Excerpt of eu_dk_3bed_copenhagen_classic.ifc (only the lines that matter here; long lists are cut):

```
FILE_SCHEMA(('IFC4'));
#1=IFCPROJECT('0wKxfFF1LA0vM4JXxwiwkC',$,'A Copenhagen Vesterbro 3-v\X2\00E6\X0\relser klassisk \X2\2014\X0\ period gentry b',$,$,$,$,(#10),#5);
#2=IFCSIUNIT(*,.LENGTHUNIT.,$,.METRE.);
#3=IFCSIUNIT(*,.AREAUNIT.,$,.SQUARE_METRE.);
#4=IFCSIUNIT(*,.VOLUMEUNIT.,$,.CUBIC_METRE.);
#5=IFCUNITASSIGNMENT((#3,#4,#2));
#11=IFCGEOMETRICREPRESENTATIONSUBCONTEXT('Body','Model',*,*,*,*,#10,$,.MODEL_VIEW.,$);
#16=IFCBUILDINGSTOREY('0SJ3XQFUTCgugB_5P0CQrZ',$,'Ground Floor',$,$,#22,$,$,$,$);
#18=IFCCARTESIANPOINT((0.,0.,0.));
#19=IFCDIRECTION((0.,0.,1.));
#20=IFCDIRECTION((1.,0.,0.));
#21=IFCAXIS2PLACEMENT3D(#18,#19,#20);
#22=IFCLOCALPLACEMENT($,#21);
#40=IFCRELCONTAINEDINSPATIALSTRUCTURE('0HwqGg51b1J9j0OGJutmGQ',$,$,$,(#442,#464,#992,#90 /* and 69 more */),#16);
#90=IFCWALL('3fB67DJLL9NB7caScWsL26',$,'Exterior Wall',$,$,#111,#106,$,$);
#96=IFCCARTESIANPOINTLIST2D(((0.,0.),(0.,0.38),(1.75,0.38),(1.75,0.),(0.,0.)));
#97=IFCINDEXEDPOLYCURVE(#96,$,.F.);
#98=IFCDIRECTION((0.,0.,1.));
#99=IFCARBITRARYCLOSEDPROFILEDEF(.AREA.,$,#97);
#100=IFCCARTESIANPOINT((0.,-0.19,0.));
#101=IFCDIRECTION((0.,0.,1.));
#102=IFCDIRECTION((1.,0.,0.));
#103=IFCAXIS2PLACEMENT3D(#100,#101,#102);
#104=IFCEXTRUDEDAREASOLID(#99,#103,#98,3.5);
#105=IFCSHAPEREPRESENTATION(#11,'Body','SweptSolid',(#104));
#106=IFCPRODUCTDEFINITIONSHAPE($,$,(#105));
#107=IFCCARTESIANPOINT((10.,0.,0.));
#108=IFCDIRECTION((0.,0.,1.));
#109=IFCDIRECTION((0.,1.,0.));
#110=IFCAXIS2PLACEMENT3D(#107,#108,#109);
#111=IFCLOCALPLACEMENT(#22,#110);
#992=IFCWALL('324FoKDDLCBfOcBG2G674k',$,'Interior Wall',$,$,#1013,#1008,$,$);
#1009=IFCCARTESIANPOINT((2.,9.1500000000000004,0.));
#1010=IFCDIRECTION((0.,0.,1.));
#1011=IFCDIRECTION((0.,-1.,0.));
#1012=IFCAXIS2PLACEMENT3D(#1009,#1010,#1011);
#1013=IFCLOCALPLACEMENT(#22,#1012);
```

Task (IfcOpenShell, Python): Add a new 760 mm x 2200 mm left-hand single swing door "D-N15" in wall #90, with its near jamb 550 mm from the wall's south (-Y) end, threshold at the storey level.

```python
import numpy as np
import ifcopenshell
import ifcopenshell.api.feature
import ifcopenshell.api.geometry
import ifcopenshell.api.root
import ifcopenshell.api.spatial
import ifcopenshell.geom
import ifcopenshell.util.element
import ifcopenshell.util.placement
import ifcopenshell.util.representation
import ifcopenshell.util.shape
import ifcopenshell.util.unit

model = ifcopenshell.open("eu_dk_3bed_copenhagen_classic.ifc")
unit_scale = ifcopenshell.util.unit.calculate_unit_scale(model)
settings = ifcopenshell.geom.settings()


def volume(element):
    """Net volume in cubic metres, openings subtracted."""
    shape = ifcopenshell.geom.create_shape(settings, element)
    return ifcopenshell.util.shape.get_volume(shape.geometry)


wall = model.by_id(90)
storey = ifcopenshell.util.element.get_container(wall, ifc_class="IfcBuildingStorey")
context = ifcopenshell.util.representation.get_context(model, "Model", "Body", "MODEL_VIEW")
before = volume(wall)

width, height, from_end, sill = 0.76, 2.2, 0.55, 0.0  # metres

# The wall runs along its own X axis, and the end named is its -X end.
wall_shape = ifcopenshell.geom.create_shape(settings, wall)
x, y, z = ifcopenshell.util.shape.get_vertices(wall_shape.geometry).T
start = x.min() + from_end
face, thickness = float(y.min()), float(y.max() - y.min())
wall_matrix = ifcopenshell.util.placement.get_local_placement(wall.ObjectPlacement)
level = ifcopenshell.util.placement.get_local_placement(storey.ObjectPlacement)[2, 3]


def in_wall(x, y):
    """Placement at x, y metres in the wall's axes, at sill height."""
    matrix = wall_matrix.copy()
    matrix[:, 3] = wall_matrix @ np.array([x / unit_scale, y / unit_scale, 0.0, 1.0])
    matrix[2, 3] = level + sill / unit_scale
    return matrix


# Opening: a box that overshoots both wall faces by 50 mm.
opening = ifcopenshell.api.root.create_entity(model, ifc_class="IfcOpeningElement", predefined_type="OPENING")
box = ifcopenshell.api.geometry.add_wall_representation(
    model, context=context, length=width, height=height, thickness=thickness + 0.1
)
ifcopenshell.api.geometry.assign_representation(model, product=opening, representation=box)
ifcopenshell.api.geometry.edit_object_placement(model, product=opening, matrix=in_wall(start, face - 0.05), is_si=False)
ifcopenshell.api.feature.add_feature(model, feature=opening, element=wall)

door = ifcopenshell.api.root.create_entity(model, ifc_class="IfcDoor", name="D-N15", predefined_type="DOOR")
door.OverallWidth, door.OverallHeight = width / unit_scale, height / unit_scale
door.OperationType = "SINGLE_SWING_LEFT"
body = ifcopenshell.api.geometry.add_door_representation(
    model,
    context=context,
    overall_width=door.OverallWidth,
    overall_height=door.OverallHeight,
    operation_type="SINGLE_SWING_LEFT",
    lining_properties={"LiningDepth": thickness / unit_scale, "ThresholdDepth": thickness / unit_scale},
)
ifcopenshell.api.geometry.assign_representation(model, product=door, representation=body)
ifcopenshell.api.spatial.assign_container(model, products=[door], relating_structure=storey)
ifcopenshell.api.feature.add_filling(model, opening=opening, element=door)

# The lining spans the wall, so the door starts at the wall face.
ifcopenshell.api.geometry.edit_object_placement(model, product=door, matrix=in_wall(start, face), is_si=False)

after = volume(wall)

print(f"wall volume {before:.3f} -> {after:.3f} m3")

model.write("eu_dk_3bed_copenhagen_classic_v2.ifc")
```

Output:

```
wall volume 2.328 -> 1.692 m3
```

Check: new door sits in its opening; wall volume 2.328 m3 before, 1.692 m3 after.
